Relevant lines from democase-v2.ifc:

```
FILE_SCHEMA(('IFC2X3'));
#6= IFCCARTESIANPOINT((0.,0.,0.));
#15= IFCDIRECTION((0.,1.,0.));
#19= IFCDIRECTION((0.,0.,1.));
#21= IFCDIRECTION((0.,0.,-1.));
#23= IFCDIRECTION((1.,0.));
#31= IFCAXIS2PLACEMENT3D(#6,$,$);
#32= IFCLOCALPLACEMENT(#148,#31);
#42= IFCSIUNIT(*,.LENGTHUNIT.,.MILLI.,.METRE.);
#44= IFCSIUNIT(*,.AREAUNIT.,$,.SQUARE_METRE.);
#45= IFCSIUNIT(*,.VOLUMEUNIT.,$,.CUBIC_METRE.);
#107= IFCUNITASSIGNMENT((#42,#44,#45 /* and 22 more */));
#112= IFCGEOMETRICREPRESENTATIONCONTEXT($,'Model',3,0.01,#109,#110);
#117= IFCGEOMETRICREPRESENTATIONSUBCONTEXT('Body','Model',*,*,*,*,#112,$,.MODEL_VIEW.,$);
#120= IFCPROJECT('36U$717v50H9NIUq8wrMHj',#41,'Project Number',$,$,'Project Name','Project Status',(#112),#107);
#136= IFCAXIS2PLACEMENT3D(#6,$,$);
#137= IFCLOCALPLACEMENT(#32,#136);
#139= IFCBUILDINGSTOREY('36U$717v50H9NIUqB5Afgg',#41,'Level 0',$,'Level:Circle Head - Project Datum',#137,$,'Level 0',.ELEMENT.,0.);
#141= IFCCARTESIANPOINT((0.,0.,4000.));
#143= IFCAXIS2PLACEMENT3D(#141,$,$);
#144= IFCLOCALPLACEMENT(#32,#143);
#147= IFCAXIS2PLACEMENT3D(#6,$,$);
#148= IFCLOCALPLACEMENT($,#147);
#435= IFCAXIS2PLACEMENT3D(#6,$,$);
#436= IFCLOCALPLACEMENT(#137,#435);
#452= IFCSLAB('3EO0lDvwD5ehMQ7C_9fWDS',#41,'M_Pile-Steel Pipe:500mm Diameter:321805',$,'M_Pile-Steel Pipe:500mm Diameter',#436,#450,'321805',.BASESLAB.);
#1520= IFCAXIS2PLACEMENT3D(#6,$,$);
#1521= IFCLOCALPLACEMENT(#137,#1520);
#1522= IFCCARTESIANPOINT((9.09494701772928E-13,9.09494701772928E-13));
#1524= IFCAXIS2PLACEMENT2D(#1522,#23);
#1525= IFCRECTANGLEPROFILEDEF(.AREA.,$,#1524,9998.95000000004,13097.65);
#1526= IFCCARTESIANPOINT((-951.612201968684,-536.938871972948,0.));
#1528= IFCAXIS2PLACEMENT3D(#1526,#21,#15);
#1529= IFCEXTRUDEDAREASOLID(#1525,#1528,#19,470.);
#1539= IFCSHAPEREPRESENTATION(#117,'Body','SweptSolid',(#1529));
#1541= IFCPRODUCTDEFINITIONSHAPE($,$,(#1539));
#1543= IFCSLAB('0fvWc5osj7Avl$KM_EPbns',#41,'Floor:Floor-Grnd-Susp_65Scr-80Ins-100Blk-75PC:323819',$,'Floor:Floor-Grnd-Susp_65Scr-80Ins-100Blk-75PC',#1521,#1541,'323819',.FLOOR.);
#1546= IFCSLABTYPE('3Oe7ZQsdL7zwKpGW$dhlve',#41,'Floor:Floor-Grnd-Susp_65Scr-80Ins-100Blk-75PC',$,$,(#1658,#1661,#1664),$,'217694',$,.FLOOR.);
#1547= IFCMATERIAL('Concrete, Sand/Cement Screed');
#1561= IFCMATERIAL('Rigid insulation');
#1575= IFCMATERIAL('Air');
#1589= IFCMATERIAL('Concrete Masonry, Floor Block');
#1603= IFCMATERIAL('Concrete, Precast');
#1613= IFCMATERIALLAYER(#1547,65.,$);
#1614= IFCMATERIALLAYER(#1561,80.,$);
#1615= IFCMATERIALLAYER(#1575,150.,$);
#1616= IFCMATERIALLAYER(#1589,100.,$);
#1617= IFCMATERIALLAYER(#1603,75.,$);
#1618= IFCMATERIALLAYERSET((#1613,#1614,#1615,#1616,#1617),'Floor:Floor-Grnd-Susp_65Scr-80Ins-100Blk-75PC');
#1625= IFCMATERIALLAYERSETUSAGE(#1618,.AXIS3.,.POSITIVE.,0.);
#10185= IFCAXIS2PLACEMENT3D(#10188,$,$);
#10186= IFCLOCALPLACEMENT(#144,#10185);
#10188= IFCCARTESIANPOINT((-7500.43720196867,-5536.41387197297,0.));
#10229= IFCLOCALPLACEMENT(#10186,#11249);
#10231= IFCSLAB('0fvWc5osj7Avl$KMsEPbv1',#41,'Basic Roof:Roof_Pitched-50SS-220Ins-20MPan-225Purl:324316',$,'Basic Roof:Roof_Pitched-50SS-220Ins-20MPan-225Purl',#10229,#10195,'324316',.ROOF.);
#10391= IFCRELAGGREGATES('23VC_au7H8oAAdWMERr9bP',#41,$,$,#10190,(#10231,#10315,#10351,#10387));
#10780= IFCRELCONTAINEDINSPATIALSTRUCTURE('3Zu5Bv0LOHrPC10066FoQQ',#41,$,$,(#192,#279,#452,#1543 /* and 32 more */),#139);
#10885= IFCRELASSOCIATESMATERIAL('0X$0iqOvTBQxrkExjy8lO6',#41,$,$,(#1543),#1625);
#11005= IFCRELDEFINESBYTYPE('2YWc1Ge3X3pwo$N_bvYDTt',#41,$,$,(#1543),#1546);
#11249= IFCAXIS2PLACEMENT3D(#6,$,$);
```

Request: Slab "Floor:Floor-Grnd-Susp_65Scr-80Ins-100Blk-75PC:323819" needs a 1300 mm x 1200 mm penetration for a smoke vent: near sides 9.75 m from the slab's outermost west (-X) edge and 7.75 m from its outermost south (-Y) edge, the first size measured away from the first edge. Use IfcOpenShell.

```python
import numpy as np
import ifcopenshell
import ifcopenshell.api.feature
import ifcopenshell.api.geometry
import ifcopenshell.api.root
import ifcopenshell.geom
import ifcopenshell.util.placement
import ifcopenshell.util.representation
import ifcopenshell.util.shape
import ifcopenshell.util.unit

model = ifcopenshell.open("democase-v2.ifc")
unit_scale = ifcopenshell.util.unit.calculate_unit_scale(model)
settings = ifcopenshell.geom.settings()


def volume(element):
    """Net volume in cubic metres, openings subtracted."""
    shape = ifcopenshell.geom.create_shape(settings, element)
    return ifcopenshell.util.shape.get_volume(shape.geometry)


slab = model.by_guid("0fvWc5osj7Avl$KM_EPbns")
before = volume(slab)

# Extent in the slab's own axes, in metres. The edges named are its -X and -Y sides.
slab_shape = ifcopenshell.geom.create_shape(settings, slab)
vertices = ifcopenshell.util.shape.get_vertices(slab_shape.geometry)
x_min, y_min, bottom = vertices.min(axis=0)
top = vertices[:, 2].max()

opening = ifcopenshell.api.root.create_entity(model, ifc_class="IfcOpeningElement", name="Smoke vent opening")
context = ifcopenshell.util.representation.get_context(model, "Model", "Body", "MODEL_VIEW")
width, depth = 1.3, 1.2
outline = [(0.0, 0.0), (width, 0.0), (width, depth), (0.0, depth), (0.0, 0.0)]
# Overshoot both faces by 50 mm so the cut is clean.
shape = ifcopenshell.api.geometry.add_slab_representation(
    model, context=context, depth=top - bottom + 0.1, polyline=outline
)
ifcopenshell.api.geometry.assign_representation(model, product=opening, representation=shape)

matrix = ifcopenshell.util.placement.get_local_placement(slab.ObjectPlacement)
matrix[:, 3] = matrix @ np.append(np.array([x_min + 9.75, y_min + 7.75, bottom - 0.05]) / unit_scale, 1.0)
ifcopenshell.api.geometry.edit_object_placement(model, product=opening, matrix=matrix, is_si=False)
ifcopenshell.api.feature.add_feature(model, feature=opening, element=slab)

after = volume(slab)

print(f"slab volume {before:.3f} -> {after:.3f} m3")

model.write("democase-v2_rev.ifc")
```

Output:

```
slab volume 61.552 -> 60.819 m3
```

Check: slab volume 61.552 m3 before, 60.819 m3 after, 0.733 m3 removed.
